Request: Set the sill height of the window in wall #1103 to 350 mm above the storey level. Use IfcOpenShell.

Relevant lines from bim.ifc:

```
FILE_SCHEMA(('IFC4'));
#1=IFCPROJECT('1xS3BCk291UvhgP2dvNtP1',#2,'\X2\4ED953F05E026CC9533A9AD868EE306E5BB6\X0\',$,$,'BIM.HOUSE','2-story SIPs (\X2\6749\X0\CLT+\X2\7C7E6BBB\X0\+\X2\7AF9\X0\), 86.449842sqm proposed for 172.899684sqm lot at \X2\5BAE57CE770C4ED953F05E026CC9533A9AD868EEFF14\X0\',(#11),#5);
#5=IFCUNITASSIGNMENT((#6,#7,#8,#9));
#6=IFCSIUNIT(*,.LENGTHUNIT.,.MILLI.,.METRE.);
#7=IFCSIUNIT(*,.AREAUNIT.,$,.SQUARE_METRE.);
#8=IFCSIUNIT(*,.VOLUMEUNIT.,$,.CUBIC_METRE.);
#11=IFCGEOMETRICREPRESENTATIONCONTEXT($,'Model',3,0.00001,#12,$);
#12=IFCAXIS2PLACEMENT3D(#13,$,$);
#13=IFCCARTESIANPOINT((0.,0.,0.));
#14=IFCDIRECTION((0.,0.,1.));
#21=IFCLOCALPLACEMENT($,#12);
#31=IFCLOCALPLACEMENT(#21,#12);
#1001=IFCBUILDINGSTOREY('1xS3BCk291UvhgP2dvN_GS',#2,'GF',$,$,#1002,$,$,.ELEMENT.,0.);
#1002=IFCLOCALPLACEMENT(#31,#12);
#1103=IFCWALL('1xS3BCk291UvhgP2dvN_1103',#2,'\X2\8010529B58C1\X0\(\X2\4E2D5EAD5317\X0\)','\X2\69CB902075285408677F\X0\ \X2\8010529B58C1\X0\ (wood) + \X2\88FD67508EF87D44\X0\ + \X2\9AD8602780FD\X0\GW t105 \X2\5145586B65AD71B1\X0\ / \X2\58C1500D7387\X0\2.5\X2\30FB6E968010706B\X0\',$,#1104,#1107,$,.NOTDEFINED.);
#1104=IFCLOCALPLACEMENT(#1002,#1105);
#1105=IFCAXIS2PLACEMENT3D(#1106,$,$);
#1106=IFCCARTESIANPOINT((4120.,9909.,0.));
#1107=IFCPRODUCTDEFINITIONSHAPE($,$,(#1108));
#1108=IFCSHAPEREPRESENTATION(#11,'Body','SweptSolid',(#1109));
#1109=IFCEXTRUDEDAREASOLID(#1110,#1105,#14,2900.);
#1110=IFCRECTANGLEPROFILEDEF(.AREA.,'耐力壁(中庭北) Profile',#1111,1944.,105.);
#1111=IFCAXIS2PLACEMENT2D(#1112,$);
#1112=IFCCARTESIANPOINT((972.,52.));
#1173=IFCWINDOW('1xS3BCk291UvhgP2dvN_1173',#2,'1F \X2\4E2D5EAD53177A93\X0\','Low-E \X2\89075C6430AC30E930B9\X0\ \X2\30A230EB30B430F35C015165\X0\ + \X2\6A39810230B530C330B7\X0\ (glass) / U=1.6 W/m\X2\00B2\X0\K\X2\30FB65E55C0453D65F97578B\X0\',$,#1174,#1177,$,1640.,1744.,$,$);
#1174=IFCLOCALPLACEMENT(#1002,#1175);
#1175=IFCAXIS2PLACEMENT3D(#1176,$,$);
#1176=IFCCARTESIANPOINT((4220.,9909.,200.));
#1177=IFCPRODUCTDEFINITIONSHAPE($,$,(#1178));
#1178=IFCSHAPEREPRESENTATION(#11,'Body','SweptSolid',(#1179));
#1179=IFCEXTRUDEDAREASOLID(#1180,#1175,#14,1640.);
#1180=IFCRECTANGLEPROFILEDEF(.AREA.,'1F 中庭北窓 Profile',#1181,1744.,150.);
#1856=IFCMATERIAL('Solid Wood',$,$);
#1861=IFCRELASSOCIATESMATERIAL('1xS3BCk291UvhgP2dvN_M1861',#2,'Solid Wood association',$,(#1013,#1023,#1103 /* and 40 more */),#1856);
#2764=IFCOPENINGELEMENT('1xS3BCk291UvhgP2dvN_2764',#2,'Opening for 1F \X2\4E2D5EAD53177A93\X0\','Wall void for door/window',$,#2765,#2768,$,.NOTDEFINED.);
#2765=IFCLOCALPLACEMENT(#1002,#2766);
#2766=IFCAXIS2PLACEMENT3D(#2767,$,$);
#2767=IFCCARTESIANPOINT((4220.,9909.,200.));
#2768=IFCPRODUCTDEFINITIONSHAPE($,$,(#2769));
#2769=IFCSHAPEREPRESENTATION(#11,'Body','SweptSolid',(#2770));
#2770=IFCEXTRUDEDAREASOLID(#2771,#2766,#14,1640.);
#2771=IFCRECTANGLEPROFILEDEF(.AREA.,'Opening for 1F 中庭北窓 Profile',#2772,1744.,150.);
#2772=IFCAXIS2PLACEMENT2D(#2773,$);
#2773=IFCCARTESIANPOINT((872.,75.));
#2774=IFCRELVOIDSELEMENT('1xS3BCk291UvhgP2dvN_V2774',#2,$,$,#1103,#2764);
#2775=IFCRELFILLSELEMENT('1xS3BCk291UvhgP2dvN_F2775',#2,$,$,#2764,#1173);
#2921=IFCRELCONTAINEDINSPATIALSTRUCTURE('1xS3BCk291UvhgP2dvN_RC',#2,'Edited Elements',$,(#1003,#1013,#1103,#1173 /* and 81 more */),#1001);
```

```python
import numpy as np
import ifcopenshell
import ifcopenshell.api.geometry
import ifcopenshell.geom
import ifcopenshell.util.element
import ifcopenshell.util.placement
import ifcopenshell.util.shape
import ifcopenshell.util.unit

model = ifcopenshell.open("bim.ifc")
unit_scale = ifcopenshell.util.unit.calculate_unit_scale(model)

window = model.by_guid("1xS3BCk291UvhgP2dvN_1173")
opening = window.FillsVoids[0].RelatingOpeningElement
storey = ifcopenshell.util.element.get_container(window, ifc_class="IfcBuildingStorey")
level = ifcopenshell.util.placement.get_local_placement(storey.ObjectPlacement)[2, 3]

# The opening's origin need not be at the sill, so measure its lowest point.
shape = ifcopenshell.geom.create_shape(ifcopenshell.geom.settings(), opening)
bottom = ifcopenshell.util.shape.get_shape_bottom_elevation(shape, shape.geometry) / unit_scale
dz = level + 350.0 - bottom

shift = np.array([0.0, 0.0, dz])
# The window is not placed relative to its opening, so move both.
for product in (opening, window):
    matrix = ifcopenshell.util.placement.get_local_placement(product.ObjectPlacement)
    matrix[:3, 3] += shift
    ifcopenshell.api.geometry.edit_object_placement(model, product=product, matrix=matrix, is_si=False)

print(f"moved by {dz * unit_scale:+.3f} m")

model.write("bim_v2.ifc")
```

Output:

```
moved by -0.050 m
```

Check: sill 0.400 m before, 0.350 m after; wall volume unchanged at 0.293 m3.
